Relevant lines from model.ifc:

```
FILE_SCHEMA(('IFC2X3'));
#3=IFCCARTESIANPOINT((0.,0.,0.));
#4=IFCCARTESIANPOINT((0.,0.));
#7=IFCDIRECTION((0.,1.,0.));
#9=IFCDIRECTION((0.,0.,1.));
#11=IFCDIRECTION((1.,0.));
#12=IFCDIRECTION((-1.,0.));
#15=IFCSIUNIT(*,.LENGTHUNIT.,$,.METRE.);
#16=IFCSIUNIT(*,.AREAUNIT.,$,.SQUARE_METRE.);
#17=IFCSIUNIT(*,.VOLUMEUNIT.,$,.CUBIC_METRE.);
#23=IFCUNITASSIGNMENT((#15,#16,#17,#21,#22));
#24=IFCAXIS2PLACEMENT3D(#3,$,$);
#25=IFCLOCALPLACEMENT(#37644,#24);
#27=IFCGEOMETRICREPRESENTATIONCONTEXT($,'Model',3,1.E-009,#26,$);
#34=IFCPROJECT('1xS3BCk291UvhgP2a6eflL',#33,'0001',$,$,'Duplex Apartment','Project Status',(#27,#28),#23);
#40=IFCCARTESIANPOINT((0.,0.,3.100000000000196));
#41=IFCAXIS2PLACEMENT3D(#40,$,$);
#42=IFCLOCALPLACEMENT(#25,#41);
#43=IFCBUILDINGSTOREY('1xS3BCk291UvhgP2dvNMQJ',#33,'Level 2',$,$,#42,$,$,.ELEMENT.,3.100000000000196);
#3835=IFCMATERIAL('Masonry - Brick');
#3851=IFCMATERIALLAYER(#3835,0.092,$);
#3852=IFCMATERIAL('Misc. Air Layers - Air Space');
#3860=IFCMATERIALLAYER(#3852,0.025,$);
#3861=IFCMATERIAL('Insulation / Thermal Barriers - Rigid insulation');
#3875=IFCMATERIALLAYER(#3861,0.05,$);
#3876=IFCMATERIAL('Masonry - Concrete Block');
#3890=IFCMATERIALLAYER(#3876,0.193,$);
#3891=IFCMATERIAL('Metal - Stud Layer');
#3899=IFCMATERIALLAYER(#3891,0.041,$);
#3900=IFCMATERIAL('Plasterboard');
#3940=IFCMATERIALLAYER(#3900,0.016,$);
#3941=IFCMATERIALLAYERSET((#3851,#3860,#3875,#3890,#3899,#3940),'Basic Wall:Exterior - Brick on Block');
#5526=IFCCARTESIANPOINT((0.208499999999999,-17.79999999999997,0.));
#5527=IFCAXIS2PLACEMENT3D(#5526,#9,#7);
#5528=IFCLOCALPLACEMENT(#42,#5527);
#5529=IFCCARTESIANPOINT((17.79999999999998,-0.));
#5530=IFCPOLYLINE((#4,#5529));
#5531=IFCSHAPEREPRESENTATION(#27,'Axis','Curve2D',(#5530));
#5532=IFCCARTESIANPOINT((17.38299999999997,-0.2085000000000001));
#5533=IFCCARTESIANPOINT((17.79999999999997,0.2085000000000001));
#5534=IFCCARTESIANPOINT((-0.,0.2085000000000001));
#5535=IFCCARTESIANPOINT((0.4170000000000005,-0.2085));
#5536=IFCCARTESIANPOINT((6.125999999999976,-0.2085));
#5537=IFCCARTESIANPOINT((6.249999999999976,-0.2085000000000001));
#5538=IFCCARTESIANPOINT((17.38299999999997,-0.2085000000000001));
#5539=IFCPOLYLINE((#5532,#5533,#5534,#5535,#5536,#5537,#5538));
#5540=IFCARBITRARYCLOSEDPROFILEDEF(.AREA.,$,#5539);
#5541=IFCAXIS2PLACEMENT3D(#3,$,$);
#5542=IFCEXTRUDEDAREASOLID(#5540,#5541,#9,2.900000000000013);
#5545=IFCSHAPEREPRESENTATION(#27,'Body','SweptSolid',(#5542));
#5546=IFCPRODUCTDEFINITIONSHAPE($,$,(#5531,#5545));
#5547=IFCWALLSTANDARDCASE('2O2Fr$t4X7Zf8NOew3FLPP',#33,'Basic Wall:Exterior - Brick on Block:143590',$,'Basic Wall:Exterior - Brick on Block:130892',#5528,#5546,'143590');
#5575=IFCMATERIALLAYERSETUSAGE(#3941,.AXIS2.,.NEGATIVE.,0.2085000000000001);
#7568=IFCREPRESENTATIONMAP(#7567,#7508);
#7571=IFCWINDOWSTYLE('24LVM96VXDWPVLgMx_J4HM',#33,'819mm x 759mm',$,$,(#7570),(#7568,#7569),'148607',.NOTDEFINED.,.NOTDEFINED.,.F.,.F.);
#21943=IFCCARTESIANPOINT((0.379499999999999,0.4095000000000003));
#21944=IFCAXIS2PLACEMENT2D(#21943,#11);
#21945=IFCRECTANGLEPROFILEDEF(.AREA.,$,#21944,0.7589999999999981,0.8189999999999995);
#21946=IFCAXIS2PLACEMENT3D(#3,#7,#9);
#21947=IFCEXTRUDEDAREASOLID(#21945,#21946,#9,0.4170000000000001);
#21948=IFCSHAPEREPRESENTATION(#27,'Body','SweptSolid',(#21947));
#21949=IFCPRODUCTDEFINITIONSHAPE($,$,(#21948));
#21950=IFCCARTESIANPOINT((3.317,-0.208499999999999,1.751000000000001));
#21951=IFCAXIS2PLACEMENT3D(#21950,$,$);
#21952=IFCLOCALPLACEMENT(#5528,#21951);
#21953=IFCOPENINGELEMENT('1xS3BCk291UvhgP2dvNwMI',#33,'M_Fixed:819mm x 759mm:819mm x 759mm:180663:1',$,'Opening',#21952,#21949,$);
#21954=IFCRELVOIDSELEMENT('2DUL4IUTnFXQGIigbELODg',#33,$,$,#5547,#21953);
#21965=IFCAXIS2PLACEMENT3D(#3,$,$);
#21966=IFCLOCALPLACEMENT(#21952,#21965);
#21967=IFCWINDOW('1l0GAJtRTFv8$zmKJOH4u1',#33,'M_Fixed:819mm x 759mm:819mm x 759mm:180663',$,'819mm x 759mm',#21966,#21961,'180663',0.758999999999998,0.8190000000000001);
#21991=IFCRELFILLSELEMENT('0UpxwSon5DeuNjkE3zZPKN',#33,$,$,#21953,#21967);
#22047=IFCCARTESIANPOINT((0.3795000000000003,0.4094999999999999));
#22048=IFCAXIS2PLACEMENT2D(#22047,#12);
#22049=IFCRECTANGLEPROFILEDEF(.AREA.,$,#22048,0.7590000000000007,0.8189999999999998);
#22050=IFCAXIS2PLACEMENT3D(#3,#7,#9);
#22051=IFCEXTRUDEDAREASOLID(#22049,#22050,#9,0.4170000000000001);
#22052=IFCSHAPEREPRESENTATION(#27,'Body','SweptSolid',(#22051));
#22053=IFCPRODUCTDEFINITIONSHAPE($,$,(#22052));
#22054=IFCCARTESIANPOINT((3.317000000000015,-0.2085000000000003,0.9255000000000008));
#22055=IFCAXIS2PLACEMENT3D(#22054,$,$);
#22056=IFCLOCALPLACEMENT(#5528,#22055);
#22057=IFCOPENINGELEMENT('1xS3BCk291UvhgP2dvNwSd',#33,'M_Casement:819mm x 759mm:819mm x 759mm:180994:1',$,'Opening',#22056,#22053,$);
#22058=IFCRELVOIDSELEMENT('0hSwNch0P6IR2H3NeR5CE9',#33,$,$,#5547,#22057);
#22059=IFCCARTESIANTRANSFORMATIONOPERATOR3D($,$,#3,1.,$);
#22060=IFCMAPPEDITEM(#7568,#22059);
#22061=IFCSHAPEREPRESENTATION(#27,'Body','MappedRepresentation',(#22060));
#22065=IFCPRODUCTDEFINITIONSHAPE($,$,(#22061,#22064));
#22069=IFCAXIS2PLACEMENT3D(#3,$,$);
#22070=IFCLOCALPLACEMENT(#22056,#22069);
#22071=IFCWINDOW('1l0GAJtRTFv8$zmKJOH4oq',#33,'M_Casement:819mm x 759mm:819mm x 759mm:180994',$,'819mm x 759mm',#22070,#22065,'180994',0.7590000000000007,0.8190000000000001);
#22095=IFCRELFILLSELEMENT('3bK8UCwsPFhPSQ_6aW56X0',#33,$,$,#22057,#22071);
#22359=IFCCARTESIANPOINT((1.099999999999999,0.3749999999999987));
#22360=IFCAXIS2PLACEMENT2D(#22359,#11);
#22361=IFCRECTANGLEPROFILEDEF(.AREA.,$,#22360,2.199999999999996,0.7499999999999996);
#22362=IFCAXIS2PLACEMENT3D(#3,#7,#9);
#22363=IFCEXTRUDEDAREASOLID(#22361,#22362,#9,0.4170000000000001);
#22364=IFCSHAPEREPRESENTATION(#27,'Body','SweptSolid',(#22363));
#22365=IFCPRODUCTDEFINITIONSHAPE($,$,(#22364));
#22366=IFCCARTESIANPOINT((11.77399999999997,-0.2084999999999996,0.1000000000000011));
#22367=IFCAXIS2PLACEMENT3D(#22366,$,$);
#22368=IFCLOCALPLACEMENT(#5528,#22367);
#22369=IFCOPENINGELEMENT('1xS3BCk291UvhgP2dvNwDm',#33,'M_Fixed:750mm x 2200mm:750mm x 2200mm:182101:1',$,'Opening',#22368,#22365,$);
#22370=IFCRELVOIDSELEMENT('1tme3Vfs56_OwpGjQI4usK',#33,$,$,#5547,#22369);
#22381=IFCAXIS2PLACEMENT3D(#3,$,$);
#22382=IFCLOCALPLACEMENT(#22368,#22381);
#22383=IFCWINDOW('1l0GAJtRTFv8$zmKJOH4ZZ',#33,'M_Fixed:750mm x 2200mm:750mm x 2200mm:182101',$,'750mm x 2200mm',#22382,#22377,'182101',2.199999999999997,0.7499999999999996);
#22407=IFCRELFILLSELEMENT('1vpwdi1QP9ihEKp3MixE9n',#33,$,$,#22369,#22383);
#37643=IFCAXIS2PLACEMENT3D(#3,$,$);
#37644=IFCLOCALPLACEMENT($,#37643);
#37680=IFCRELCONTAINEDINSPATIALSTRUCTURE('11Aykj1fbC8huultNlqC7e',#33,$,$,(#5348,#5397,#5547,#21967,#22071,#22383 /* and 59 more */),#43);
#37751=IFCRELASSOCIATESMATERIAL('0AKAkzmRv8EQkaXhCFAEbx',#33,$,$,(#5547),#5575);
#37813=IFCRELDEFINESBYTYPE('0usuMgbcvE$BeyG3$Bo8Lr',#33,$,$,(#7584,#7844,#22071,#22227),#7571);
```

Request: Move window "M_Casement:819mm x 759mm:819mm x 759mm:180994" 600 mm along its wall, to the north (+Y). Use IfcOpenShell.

```python
import ifcopenshell
import ifcopenshell.api.geometry
import ifcopenshell.util.placement

model = ifcopenshell.open("model.ifc")

window = model.by_guid("1l0GAJtRTFv8$zmKJOH4oq")
opening = window.FillsVoids[0].RelatingOpeningElement
wall = opening.VoidsElements[0].RelatingBuildingElement

wall_matrix = ifcopenshell.util.placement.get_local_placement(wall.ObjectPlacement)
shift = wall_matrix[:3, 0] * 0.6
before = ifcopenshell.util.placement.get_local_placement(window.ObjectPlacement)[:3, 3].copy()

# The window is placed relative to its opening, so it follows when the opening moves.
matrix = ifcopenshell.util.placement.get_local_placement(opening.ObjectPlacement)
matrix[:3, 3] += shift
ifcopenshell.api.geometry.edit_object_placement(
    model, product=opening, matrix=matrix, is_si=False, should_transform_children=True
)

after = ifcopenshell.util.placement.get_local_placement(window.ObjectPlacement)[:3, 3]
print("window moved by", (after - before).round(3) + 0.0)

model.write("model_edited.ifc")
```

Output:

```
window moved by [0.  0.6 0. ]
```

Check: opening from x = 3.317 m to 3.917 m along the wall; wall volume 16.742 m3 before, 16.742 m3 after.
